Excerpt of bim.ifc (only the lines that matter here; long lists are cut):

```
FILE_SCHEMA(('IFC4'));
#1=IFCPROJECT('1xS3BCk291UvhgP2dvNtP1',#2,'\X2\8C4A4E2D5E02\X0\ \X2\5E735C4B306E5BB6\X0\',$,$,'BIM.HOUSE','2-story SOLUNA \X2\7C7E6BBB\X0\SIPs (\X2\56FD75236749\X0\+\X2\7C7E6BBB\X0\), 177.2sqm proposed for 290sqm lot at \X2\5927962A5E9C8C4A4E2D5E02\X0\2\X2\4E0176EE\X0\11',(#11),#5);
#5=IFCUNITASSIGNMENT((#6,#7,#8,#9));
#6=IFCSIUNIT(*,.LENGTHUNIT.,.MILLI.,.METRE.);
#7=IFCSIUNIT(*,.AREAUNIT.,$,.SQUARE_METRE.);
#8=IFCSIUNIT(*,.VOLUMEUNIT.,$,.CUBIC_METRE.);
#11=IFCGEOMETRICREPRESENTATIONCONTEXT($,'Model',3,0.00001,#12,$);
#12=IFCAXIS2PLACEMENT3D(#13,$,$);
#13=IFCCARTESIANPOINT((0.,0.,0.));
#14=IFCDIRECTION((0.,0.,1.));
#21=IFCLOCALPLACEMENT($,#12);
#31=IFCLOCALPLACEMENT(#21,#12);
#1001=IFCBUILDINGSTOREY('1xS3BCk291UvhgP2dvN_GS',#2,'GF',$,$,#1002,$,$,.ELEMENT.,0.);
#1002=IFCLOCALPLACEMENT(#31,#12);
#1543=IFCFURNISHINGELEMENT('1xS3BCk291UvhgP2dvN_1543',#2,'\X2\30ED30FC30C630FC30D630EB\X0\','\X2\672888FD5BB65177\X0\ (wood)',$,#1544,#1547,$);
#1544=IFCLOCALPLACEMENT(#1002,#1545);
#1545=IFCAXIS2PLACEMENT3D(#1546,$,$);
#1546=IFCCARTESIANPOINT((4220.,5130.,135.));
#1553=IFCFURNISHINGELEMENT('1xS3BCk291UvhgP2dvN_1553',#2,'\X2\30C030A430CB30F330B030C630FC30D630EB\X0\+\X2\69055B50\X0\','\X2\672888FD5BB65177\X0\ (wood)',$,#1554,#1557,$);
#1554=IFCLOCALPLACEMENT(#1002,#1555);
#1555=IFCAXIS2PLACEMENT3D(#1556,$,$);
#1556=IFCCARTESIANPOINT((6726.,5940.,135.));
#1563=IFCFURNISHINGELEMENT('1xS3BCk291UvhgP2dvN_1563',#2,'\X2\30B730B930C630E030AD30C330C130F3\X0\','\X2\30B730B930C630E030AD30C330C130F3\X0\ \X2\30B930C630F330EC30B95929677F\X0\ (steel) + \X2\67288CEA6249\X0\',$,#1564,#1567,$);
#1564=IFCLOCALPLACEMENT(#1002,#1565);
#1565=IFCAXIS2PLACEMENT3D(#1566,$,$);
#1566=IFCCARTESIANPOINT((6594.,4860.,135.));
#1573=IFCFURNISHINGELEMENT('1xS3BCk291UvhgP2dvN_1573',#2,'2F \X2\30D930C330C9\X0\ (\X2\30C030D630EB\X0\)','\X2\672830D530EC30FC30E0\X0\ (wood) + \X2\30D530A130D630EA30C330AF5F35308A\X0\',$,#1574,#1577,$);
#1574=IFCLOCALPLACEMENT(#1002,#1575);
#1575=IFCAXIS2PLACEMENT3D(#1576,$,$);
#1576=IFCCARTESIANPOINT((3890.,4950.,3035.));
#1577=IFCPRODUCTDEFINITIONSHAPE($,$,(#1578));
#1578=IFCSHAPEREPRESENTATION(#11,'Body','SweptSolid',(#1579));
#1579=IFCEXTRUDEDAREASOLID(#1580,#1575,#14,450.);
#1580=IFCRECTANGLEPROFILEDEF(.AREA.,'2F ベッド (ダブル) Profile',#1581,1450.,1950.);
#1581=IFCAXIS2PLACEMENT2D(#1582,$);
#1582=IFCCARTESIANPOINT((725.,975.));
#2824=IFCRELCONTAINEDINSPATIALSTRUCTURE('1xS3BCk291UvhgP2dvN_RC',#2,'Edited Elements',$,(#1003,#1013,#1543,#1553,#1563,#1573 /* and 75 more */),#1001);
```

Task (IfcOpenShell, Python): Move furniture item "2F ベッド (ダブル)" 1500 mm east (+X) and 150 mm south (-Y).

```python
import ifcopenshell
import ifcopenshell.api.geometry
import ifcopenshell.util.placement
import ifcopenshell.util.unit

model = ifcopenshell.open("bim.ifc")
unit_scale = ifcopenshell.util.unit.calculate_unit_scale(model)

item = model.by_id(1573)
matrix = ifcopenshell.util.placement.get_local_placement(item.ObjectPlacement)
matrix[0, 3] += 1.5 / unit_scale
matrix[1, 3] -= 0.15 / unit_scale
ifcopenshell.api.geometry.edit_object_placement(model, product=item, matrix=matrix, is_si=False)

print(ifcopenshell.util.placement.get_local_placement(item.ObjectPlacement).round(3) + 0.0)

model.write("bim_v2.ifc")
```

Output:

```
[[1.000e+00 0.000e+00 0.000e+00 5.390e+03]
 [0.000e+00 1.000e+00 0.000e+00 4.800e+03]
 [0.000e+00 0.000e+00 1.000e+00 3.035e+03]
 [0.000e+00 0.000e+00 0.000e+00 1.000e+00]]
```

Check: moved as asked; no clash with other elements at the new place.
